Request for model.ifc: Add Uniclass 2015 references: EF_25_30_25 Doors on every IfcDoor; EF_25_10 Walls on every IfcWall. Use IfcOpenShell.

First a look at what the model holds.

```python
import ifcopenshell

model = ifcopenshell.open("model.ifc")
print(model.schema)
print("classifications:", [c.Name for c in model.by_type("IfcClassification")])
for ifc_class in ("IfcDoor", "IfcRoof", "IfcStair", "IfcWall", "IfcWindow"):
    print(ifc_class, len(model.by_type(ifc_class)))
```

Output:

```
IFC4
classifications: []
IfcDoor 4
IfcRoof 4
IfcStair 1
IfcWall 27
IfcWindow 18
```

```python
import ifcopenshell
import ifcopenshell.api.classification

model = ifcopenshell.open("model.ifc")

system = ifcopenshell.api.classification.add_classification(model, classification="Uniclass 2015")

codes = {
    "IfcDoor": ("EF_25_30_25", "Doors"),
    "IfcWall": ("EF_25_10", "Walls"),
}
for ifc_class, (code, name) in codes.items():
    products = model.by_type(ifc_class)
    ifcopenshell.api.classification.add_reference(
        model, products=products, classification=system, identification=code, name=name
    )
    print(code, len(products))

model.write("model_updated.ifc")
```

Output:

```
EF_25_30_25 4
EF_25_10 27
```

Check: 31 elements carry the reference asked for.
